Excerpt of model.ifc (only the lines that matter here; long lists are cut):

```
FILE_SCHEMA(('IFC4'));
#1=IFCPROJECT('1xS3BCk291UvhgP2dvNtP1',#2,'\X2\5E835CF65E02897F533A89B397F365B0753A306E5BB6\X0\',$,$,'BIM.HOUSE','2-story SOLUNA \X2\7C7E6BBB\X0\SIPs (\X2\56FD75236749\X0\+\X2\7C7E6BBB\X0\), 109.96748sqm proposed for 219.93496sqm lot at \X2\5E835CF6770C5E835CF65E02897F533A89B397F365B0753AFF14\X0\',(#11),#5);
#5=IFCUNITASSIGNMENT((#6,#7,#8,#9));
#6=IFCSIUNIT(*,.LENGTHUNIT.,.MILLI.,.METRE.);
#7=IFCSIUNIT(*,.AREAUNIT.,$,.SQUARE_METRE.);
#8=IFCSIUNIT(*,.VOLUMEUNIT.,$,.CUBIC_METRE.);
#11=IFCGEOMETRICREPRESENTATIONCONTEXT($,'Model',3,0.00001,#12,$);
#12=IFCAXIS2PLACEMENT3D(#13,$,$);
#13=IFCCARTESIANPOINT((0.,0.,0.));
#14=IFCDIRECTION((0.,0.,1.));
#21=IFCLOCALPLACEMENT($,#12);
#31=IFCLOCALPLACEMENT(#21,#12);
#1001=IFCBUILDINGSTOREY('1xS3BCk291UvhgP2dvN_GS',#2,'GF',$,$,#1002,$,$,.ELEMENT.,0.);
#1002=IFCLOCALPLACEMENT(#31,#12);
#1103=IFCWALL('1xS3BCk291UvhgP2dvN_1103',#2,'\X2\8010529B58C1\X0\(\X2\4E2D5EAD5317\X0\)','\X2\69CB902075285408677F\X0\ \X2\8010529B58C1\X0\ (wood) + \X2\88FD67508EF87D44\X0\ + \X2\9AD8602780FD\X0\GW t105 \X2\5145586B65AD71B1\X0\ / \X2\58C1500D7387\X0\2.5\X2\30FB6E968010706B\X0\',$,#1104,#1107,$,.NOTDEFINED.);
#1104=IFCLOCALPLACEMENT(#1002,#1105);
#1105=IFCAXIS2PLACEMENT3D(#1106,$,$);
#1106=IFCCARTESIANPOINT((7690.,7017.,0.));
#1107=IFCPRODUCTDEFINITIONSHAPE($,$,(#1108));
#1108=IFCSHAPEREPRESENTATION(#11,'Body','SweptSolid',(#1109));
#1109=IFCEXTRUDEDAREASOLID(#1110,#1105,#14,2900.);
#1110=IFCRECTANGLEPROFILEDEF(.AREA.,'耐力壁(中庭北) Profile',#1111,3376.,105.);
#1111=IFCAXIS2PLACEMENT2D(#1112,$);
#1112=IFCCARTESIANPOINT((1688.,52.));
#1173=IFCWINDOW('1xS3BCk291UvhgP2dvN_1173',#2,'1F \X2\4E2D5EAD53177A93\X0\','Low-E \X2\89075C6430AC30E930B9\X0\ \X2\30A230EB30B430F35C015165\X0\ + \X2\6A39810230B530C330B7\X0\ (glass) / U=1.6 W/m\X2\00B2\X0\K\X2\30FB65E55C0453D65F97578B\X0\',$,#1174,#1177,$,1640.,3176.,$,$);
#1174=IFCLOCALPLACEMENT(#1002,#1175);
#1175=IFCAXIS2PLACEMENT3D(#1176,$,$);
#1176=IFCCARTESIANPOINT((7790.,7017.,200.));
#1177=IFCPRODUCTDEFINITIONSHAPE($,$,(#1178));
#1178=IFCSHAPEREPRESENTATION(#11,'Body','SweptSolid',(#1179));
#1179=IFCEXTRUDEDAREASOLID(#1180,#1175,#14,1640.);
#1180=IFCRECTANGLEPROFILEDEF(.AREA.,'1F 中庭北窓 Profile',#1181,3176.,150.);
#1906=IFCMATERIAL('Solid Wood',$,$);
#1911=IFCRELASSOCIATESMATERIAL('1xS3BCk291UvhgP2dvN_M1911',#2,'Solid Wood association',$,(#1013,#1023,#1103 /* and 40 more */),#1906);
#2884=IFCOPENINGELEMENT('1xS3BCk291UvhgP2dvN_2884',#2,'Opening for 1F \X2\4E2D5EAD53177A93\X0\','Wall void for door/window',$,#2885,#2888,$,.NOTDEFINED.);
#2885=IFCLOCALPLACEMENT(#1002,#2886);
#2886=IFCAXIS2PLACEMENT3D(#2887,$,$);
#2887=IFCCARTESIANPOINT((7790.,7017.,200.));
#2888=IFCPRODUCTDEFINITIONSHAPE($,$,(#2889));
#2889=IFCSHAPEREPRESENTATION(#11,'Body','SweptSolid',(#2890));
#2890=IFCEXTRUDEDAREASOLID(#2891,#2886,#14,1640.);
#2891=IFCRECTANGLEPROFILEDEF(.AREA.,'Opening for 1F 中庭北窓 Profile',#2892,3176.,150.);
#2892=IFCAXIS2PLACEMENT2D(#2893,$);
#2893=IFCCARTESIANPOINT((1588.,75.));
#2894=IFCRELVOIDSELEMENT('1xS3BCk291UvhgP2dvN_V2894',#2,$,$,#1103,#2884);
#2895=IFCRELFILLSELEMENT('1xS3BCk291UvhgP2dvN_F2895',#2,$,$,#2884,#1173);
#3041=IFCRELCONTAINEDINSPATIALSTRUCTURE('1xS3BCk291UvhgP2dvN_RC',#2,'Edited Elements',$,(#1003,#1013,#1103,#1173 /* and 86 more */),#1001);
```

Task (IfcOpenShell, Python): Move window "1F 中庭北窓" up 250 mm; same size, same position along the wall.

```python
import numpy as np
import ifcopenshell
import ifcopenshell.api.geometry
import ifcopenshell.util.placement
import ifcopenshell.util.unit

model = ifcopenshell.open("model.ifc")
unit_scale = ifcopenshell.util.unit.calculate_unit_scale(model)

window = model.by_guid("1xS3BCk291UvhgP2dvN_1173")
opening = window.FillsVoids[0].RelatingOpeningElement
dz = 0.25 / unit_scale

shift = np.array([0.0, 0.0, dz])
# The window is not placed relative to its opening, so move both.
for product in (opening, window):
    matrix = ifcopenshell.util.placement.get_local_placement(product.ObjectPlacement)
    matrix[:3, 3] += shift
    ifcopenshell.api.geometry.edit_object_placement(model, product=product, matrix=matrix, is_si=False)

print(f"moved by {dz * unit_scale:+.3f} m")

model.write("model_v2.ifc")
```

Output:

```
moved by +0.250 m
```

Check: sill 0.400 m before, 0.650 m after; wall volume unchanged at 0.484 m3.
